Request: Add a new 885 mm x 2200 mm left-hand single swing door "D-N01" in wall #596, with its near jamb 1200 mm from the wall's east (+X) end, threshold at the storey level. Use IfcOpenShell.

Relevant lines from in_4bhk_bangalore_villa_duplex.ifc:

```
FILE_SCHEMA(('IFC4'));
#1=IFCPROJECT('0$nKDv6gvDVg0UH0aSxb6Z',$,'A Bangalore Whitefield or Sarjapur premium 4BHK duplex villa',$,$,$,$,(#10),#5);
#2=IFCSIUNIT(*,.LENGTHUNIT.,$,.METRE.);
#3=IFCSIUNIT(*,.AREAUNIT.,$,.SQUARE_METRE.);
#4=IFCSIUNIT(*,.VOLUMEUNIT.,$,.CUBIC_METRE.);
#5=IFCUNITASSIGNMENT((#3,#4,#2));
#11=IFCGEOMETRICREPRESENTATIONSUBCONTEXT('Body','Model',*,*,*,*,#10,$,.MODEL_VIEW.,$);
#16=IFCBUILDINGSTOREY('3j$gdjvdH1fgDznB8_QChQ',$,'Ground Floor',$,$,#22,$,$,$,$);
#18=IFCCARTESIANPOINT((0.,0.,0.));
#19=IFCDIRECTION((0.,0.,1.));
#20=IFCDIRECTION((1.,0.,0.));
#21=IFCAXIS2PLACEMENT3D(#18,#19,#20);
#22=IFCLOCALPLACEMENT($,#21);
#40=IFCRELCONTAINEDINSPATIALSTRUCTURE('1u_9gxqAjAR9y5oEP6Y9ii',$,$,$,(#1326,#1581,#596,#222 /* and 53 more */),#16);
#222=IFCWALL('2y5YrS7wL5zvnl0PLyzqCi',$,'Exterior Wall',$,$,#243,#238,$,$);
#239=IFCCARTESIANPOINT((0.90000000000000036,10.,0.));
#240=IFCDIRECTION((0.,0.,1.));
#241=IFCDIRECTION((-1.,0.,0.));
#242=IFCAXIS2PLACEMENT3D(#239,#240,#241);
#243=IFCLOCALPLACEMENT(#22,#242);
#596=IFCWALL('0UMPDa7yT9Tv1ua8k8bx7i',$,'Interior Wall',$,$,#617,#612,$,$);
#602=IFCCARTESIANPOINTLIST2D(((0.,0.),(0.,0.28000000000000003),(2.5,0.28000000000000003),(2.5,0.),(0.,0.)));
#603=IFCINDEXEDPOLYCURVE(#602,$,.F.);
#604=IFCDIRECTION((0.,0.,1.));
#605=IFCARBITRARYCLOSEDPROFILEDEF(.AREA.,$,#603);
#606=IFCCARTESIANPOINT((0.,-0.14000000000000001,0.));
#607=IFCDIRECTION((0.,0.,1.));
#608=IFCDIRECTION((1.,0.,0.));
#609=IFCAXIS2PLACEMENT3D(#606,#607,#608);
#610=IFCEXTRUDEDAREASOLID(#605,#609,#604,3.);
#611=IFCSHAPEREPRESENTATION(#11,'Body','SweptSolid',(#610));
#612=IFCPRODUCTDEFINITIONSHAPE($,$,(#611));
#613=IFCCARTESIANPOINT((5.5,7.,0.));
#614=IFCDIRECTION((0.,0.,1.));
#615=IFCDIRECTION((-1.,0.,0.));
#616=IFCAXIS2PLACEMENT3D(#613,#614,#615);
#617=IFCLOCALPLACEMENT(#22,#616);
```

```python
import numpy as np
import ifcopenshell
import ifcopenshell.api.feature
import ifcopenshell.api.geometry
import ifcopenshell.api.root
import ifcopenshell.api.spatial
import ifcopenshell.geom
import ifcopenshell.util.element
import ifcopenshell.util.placement
import ifcopenshell.util.representation
import ifcopenshell.util.shape
import ifcopenshell.util.unit

model = ifcopenshell.open("in_4bhk_bangalore_villa_duplex.ifc")
unit_scale = ifcopenshell.util.unit.calculate_unit_scale(model)
settings = ifcopenshell.geom.settings()


def volume(element):
    """Net volume in cubic metres, openings subtracted."""
    shape = ifcopenshell.geom.create_shape(settings, element)
    return ifcopenshell.util.shape.get_volume(shape.geometry)


wall = model.by_guid("0UMPDa7yT9Tv1ua8k8bx7i")
storey = ifcopenshell.util.element.get_container(wall, ifc_class="IfcBuildingStorey")
context = ifcopenshell.util.representation.get_context(model, "Model", "Body", "MODEL_VIEW")
before = volume(wall)

width, height, from_end, sill = 0.885, 2.2, 1.2, 0.0  # metres

# The wall runs along its own X axis, and the end named is its -X end.
wall_shape = ifcopenshell.geom.create_shape(settings, wall)
x, y, z = ifcopenshell.util.shape.get_vertices(wall_shape.geometry).T
start = x.min() + from_end
face, thickness = float(y.min()), float(y.max() - y.min())
wall_matrix = ifcopenshell.util.placement.get_local_placement(wall.ObjectPlacement)
level = ifcopenshell.util.placement.get_local_placement(storey.ObjectPlacement)[2, 3]


def in_wall(x, y):
    """Placement at x, y metres in the wall's axes, at sill height."""
    matrix = wall_matrix.copy()
    matrix[:, 3] = wall_matrix @ np.array([x / unit_scale, y / unit_scale, 0.0, 1.0])
    matrix[2, 3] = level + sill / unit_scale
    return matrix


# Opening: a box that overshoots both wall faces by 50 mm.
opening = ifcopenshell.api.root.create_entity(model, ifc_class="IfcOpeningElement", predefined_type="OPENING")
box = ifcopenshell.api.geometry.add_wall_representation(
    model, context=context, length=width, height=height, thickness=thickness + 0.1
)
ifcopenshell.api.geometry.assign_representation(model, product=opening, representation=box)
ifcopenshell.api.geometry.edit_object_placement(model, product=opening, matrix=in_wall(start, face - 0.05), is_si=False)
ifcopenshell.api.feature.add_feature(model, feature=opening, element=wall)

door = ifcopenshell.api.root.create_entity(model, ifc_class="IfcDoor", name="D-N01", predefined_type="DOOR")
door.OverallWidth, door.OverallHeight = width / unit_scale, height / unit_scale
door.OperationType = "SINGLE_SWING_LEFT"
body = ifcopenshell.api.geometry.add_door_representation(
    model,
    context=context,
    overall_width=door.OverallWidth,
    overall_height=door.OverallHeight,
    operation_type="SINGLE_SWING_LEFT",
    lining_properties={"LiningDepth": thickness / unit_scale, "ThresholdDepth": thickness / unit_scale},
)
ifcopenshell.api.geometry.assign_representation(model, product=door, representation=body)
ifcopenshell.api.spatial.assign_container(model, products=[door], relating_structure=storey)
ifcopenshell.api.feature.add_filling(model, opening=opening, element=door)

# The lining spans the wall, so the door starts at the wall face.
ifcopenshell.api.geometry.edit_object_placement(model, product=door, matrix=in_wall(start, face), is_si=False)

after = volume(wall)

print(f"wall volume {before:.3f} -> {after:.3f} m3")

model.write("in_4bhk_bangalore_villa_duplex_v2.ifc")
```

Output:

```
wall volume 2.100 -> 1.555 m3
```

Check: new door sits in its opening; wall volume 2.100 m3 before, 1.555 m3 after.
